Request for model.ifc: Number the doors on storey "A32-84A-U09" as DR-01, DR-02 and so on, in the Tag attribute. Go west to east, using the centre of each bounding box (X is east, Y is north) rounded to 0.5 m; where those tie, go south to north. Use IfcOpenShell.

First a look at what the model holds.

```python
import ifcopenshell
import ifcopenshell.util.element
import ifcopenshell.util.placement

model = ifcopenshell.open("model.ifc")
print(model.schema)
storey = next(s for s in model.by_type("IfcBuildingStorey") if s.Name == "A32-84A-U09")
doors = [e for e in ifcopenshell.util.element.get_decomposition(storey) if e.is_a("IfcDoor")]
for e in sorted(doors, key=lambda e: e.id()):
    origin = ifcopenshell.util.placement.get_local_placement(e.ObjectPlacement)[:3, 3]
    print(e.id(), e.Tag, e.Name, origin.round(2) + 0.0, sep=" | ")
```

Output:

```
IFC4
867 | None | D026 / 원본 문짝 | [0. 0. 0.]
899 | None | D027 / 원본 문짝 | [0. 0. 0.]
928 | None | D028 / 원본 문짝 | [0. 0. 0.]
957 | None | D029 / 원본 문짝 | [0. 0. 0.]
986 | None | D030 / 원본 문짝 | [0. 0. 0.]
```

```python
import ifcopenshell
import ifcopenshell.geom
import ifcopenshell.util.element
import ifcopenshell.util.shape

model = ifcopenshell.open("model.ifc")
settings = ifcopenshell.geom.settings()
settings.set("use-world-coords", True)


def centre(element):
    shape = ifcopenshell.geom.create_shape(settings, element)
    return ifcopenshell.util.shape.get_bbox_centroid(shape.geometry)


storey = next(s for s in model.by_type("IfcBuildingStorey") if s.Name == "A32-84A-U09")
doors = [e for e in ifcopenshell.util.element.get_decomposition(storey) if e.is_a("IfcDoor")]

# Insertion points can sit at a corner or the storey origin, so sort by the geometry (in metres).
centres = {e: centre(e) for e in doors}
doors.sort(key=lambda e: (round(centres[e][0] / 0.5), centres[e][1]))

for i, e in enumerate(doors, start=1):
    number = f"DR-{i:02d}"
    e.Tag = number
    print(e.id(), number)

model.write("model_edited.ifc")
```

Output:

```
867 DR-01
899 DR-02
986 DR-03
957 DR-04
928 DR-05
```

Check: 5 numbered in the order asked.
